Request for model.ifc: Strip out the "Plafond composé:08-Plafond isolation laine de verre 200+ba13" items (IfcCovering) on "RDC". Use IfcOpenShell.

First a look at what the model holds.

```python
import ifcopenshell
import ifcopenshell.util.element

model = ifcopenshell.open("model.ifc")
print(model.schema)
storey = next(s for s in model.by_type("IfcBuildingStorey") if s.Name == "RDC")
coverings = [e for e in ifcopenshell.util.element.get_decomposition(storey) if e.is_a("IfcCovering")]
seen = {}
for e in coverings:
    element_type = ifcopenshell.util.element.get_type(e)
    name = element_type.Name if element_type not in (None, e) else None
    seen[name] = seen.get(name, 0) + 1
for name, count in sorted(seen.items(), key=str):
    print(count, "x", name)
```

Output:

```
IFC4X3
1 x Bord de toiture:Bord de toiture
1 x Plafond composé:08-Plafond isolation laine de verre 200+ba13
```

```python
import ifcopenshell
import ifcopenshell.api.root
import ifcopenshell.util.element

model = ifcopenshell.open("model.ifc")

storey = next(s for s in model.by_type("IfcBuildingStorey") if s.Name == "RDC")
coverings = [e for e in ifcopenshell.util.element.get_decomposition(storey) if e.is_a("IfcCovering")]
targets = [e for e in coverings if (t := ifcopenshell.util.element.get_type(e)) not in (None, e) and t.Name == "Plafond composé:08-Plafond isolation laine de verre 200+ba13"]

for e in targets:
    ifcopenshell.api.root.remove_product(model, product=e)
print(len(targets), "removed")

model.write("model_rev.ifc")
```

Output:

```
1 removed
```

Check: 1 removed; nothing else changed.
